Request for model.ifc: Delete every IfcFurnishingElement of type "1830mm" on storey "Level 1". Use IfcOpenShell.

First a look at what the model holds.

```python
import ifcopenshell
import ifcopenshell.util.element

model = ifcopenshell.open("model.ifc")
print(model.schema)
storey = next(s for s in model.by_type("IfcBuildingStorey") if s.Name == "Level 1")
furniture = [e for e in ifcopenshell.util.element.get_decomposition(storey) if e.is_a("IfcFurnishingElement")]
seen = {}
for e in furniture:
    element_type = ifcopenshell.util.element.get_type(e)
    name = element_type.Name if element_type not in (None, e) else None
    seen[name] = seen.get(name, 0) + 1
for name, count in sorted(seen.items(), key=str):
    print(count, "x", name)
```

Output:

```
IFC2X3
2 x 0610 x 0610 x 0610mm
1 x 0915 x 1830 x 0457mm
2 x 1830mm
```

```python
import ifcopenshell
import ifcopenshell.api.root
import ifcopenshell.util.element

model = ifcopenshell.open("model.ifc")

storey = next(s for s in model.by_type("IfcBuildingStorey") if s.Name == "Level 1")
furniture = [e for e in ifcopenshell.util.element.get_decomposition(storey) if e.is_a("IfcFurnishingElement")]
targets = [e for e in furniture if (t := ifcopenshell.util.element.get_type(e)) not in (None, e) and t.Name == "1830mm"]

for e in targets:
    ifcopenshell.api.root.remove_product(model, product=e)
print(len(targets), "removed")

model.write("model_edited.ifc")
```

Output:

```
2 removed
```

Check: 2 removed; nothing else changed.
